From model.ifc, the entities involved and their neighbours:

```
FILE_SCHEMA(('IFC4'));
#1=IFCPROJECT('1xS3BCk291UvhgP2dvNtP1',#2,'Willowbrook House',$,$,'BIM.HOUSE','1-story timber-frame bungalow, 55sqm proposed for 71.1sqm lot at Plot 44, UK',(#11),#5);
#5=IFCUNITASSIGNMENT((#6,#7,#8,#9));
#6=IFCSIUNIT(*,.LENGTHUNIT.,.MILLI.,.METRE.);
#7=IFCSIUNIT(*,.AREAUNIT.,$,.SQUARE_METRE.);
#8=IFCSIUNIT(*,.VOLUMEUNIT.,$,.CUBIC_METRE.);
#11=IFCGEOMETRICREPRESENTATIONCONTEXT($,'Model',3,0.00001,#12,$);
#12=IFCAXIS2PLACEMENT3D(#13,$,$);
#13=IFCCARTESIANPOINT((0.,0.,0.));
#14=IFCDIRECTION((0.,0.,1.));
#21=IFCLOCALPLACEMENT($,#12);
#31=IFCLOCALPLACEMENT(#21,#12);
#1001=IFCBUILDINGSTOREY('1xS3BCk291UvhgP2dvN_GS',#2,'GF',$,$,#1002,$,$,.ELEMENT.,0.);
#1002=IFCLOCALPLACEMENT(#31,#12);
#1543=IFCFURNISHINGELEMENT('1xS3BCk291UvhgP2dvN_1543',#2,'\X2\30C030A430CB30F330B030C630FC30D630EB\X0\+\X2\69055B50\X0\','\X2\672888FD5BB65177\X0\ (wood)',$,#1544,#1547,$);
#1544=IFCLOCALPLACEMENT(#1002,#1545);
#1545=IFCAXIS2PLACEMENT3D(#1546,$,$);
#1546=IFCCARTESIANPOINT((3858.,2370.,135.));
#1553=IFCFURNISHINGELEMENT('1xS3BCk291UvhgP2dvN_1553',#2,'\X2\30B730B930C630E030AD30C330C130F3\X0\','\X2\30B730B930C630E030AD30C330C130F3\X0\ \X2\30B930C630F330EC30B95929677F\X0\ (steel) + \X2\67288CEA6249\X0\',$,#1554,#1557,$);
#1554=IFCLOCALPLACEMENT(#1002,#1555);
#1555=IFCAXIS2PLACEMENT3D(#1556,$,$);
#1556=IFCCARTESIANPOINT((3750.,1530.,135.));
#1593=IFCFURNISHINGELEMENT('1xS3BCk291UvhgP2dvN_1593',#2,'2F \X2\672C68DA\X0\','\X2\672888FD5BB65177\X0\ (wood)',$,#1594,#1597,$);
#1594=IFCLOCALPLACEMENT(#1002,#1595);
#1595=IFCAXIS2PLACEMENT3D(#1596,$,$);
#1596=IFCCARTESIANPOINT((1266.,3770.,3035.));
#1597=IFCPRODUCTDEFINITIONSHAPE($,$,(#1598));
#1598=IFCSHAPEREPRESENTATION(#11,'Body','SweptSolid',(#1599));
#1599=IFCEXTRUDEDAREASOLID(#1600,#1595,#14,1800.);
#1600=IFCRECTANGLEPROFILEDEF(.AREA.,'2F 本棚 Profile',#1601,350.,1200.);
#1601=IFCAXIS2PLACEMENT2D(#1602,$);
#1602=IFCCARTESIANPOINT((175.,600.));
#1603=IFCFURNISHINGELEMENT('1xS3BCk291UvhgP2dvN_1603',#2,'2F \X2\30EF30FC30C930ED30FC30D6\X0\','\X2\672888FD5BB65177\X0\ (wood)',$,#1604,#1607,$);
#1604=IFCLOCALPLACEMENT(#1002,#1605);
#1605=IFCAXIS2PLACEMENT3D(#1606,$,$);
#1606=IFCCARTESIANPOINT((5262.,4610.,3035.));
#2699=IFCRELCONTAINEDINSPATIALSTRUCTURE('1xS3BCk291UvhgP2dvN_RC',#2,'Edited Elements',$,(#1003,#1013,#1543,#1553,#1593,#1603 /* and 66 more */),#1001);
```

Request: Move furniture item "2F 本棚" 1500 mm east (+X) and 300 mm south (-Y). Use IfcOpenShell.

```python
import ifcopenshell
import ifcopenshell.api.geometry
import ifcopenshell.util.placement

model = ifcopenshell.open("model.ifc")

item = model.by_guid("1xS3BCk291UvhgP2dvN_1593")
matrix = ifcopenshell.util.placement.get_local_placement(item.ObjectPlacement)
matrix[0, 3] += 1500.0
matrix[1, 3] -= 300.0
ifcopenshell.api.geometry.edit_object_placement(model, product=item, matrix=matrix, is_si=False)

print(ifcopenshell.util.placement.get_local_placement(item.ObjectPlacement).round(3) + 0.0)

model.write("model_v2.ifc")
```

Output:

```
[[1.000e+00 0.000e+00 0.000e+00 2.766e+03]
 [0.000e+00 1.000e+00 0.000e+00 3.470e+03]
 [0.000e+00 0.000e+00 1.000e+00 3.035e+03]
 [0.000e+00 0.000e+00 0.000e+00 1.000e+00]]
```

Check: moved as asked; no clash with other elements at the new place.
